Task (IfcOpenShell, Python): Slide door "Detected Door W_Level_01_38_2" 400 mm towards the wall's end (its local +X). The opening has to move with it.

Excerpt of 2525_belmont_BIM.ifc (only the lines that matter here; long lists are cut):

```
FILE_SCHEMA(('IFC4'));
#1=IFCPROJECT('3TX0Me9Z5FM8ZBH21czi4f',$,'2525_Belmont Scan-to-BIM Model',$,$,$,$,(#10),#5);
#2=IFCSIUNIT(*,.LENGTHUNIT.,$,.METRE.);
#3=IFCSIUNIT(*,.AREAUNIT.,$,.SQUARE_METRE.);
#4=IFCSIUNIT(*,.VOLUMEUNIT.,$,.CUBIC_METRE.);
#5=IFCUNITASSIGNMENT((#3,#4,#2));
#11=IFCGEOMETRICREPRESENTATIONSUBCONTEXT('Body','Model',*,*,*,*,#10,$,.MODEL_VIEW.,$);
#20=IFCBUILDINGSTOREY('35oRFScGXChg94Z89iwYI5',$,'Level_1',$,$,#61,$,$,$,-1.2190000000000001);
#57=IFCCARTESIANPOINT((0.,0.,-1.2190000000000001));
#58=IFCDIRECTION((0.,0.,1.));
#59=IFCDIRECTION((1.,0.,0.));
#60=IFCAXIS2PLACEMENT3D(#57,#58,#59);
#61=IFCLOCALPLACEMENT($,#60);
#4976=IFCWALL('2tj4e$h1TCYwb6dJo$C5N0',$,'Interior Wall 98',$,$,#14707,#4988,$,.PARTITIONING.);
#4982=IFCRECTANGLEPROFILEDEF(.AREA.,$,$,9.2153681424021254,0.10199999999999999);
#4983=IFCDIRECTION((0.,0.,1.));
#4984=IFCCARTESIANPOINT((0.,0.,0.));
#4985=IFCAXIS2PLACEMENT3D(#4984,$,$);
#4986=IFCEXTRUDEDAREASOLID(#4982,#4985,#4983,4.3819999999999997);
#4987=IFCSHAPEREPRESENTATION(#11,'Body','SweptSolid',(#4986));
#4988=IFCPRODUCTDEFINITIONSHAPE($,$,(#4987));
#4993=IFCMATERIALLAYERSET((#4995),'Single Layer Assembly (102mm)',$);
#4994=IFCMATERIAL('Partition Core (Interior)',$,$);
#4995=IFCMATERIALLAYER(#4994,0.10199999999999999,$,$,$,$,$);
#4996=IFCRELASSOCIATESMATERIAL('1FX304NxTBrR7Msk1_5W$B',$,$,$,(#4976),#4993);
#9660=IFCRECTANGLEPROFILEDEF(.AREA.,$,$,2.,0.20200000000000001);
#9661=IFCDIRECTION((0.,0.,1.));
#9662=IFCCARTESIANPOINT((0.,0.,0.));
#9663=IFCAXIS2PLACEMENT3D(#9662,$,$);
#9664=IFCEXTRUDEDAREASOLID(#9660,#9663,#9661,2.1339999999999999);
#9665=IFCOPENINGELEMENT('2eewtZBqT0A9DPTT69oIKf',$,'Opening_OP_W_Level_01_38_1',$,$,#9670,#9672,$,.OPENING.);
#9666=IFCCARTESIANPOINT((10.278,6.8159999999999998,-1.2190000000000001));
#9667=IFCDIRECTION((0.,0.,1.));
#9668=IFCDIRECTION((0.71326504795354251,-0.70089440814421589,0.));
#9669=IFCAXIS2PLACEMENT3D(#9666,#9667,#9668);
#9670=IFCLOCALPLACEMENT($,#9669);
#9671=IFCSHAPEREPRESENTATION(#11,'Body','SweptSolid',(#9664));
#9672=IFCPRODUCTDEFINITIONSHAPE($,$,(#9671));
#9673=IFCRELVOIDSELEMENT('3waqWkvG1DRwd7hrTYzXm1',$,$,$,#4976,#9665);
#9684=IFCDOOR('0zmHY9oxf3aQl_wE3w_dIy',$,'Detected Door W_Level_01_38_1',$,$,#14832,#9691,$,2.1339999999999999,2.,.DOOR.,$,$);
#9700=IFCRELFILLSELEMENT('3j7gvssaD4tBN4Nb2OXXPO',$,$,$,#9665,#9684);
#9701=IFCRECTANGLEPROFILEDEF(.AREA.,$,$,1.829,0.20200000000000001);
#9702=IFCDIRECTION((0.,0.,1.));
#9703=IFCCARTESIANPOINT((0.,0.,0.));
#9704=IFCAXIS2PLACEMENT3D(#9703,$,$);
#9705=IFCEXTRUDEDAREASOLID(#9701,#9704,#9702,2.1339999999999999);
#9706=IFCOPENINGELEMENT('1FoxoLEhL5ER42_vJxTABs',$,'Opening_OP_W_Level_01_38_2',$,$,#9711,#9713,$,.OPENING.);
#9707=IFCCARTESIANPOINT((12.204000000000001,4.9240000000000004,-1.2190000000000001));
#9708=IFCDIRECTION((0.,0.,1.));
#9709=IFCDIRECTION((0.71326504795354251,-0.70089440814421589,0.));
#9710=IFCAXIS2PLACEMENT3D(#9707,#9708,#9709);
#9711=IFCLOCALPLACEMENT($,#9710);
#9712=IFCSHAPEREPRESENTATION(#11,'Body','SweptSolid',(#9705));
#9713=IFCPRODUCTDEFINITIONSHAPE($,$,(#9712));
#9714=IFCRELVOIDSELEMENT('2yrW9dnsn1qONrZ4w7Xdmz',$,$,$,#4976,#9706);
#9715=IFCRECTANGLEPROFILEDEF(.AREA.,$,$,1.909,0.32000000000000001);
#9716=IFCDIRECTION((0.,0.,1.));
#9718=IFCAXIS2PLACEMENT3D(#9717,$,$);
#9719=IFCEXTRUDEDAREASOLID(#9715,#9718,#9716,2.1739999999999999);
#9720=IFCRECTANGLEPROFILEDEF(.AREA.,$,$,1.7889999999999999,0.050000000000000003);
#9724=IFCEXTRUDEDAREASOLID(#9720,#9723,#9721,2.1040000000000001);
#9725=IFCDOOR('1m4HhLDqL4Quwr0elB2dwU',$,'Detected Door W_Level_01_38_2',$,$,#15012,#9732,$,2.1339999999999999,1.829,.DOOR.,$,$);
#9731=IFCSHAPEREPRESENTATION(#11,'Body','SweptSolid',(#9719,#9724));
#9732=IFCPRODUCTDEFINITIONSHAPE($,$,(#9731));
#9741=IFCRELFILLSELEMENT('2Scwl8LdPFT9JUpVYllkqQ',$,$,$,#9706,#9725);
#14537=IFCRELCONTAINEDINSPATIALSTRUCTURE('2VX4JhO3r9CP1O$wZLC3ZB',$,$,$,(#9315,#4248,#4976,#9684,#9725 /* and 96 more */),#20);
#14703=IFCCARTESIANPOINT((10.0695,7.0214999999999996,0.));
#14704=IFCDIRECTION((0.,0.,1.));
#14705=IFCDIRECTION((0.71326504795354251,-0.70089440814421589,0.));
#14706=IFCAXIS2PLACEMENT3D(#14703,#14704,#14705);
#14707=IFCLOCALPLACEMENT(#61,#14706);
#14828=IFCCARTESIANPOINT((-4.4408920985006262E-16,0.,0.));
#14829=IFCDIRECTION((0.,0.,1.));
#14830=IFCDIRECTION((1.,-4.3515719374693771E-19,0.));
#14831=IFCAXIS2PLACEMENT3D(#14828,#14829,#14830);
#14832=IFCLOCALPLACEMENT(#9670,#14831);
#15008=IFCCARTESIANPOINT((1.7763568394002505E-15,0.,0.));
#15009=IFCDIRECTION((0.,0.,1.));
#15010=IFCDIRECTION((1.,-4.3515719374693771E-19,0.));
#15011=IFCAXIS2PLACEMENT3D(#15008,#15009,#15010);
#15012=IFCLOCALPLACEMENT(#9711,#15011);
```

```python
import ifcopenshell
import ifcopenshell.api.geometry
import ifcopenshell.util.placement
import ifcopenshell.util.unit

model = ifcopenshell.open("2525_belmont_BIM.ifc")
unit_scale = ifcopenshell.util.unit.calculate_unit_scale(model)

door = model.by_guid("1m4HhLDqL4Quwr0elB2dwU")
opening = door.FillsVoids[0].RelatingOpeningElement
wall = opening.VoidsElements[0].RelatingBuildingElement

wall_matrix = ifcopenshell.util.placement.get_local_placement(wall.ObjectPlacement)
shift = wall_matrix[:3, 0] * 0.4 / unit_scale
before = ifcopenshell.util.placement.get_local_placement(door.ObjectPlacement)[:3, 3].copy()

# The door is placed relative to its opening, so it follows when the opening moves.
matrix = ifcopenshell.util.placement.get_local_placement(opening.ObjectPlacement)
matrix[:3, 3] += shift
ifcopenshell.api.geometry.edit_object_placement(
    model, product=opening, matrix=matrix, is_si=False, should_transform_children=True
)

after = ifcopenshell.util.placement.get_local_placement(door.ObjectPlacement)[:3, 3]
print("door moved by", (after - before).round(3) + 0.0)

model.write("2525_belmont_BIM_edited.ifc")
```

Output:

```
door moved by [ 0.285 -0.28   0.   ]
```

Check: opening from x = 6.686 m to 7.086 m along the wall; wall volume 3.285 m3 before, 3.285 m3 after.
